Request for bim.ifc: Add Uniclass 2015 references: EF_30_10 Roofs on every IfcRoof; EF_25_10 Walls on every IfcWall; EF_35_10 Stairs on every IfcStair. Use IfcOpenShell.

First a look at what the model holds.

```python
import ifcopenshell

model = ifcopenshell.open("bim.ifc")
print(model.schema)
print("classifications:", [c.Name for c in model.by_type("IfcClassification")])
for ifc_class in ("IfcDoor", "IfcRoof", "IfcStair", "IfcWall", "IfcWindow"):
    print(ifc_class, len(model.by_type(ifc_class)))
```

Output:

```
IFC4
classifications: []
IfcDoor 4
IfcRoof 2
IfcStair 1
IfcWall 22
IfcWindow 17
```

```python
import ifcopenshell
import ifcopenshell.api.classification

model = ifcopenshell.open("bim.ifc")

system = ifcopenshell.api.classification.add_classification(model, classification="Uniclass 2015")

codes = {
    "IfcRoof": ("EF_30_10", "Roofs"),
    "IfcWall": ("EF_25_10", "Walls"),
    "IfcStair": ("EF_35_10", "Stairs"),
}
for ifc_class, (code, name) in codes.items():
    products = model.by_type(ifc_class)
    ifcopenshell.api.classification.add_reference(
        model, products=products, classification=system, identification=code, name=name
    )
    print(code, len(products))

model.write("bim_updated.ifc")
```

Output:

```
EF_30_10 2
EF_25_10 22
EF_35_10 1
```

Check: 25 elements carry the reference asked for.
